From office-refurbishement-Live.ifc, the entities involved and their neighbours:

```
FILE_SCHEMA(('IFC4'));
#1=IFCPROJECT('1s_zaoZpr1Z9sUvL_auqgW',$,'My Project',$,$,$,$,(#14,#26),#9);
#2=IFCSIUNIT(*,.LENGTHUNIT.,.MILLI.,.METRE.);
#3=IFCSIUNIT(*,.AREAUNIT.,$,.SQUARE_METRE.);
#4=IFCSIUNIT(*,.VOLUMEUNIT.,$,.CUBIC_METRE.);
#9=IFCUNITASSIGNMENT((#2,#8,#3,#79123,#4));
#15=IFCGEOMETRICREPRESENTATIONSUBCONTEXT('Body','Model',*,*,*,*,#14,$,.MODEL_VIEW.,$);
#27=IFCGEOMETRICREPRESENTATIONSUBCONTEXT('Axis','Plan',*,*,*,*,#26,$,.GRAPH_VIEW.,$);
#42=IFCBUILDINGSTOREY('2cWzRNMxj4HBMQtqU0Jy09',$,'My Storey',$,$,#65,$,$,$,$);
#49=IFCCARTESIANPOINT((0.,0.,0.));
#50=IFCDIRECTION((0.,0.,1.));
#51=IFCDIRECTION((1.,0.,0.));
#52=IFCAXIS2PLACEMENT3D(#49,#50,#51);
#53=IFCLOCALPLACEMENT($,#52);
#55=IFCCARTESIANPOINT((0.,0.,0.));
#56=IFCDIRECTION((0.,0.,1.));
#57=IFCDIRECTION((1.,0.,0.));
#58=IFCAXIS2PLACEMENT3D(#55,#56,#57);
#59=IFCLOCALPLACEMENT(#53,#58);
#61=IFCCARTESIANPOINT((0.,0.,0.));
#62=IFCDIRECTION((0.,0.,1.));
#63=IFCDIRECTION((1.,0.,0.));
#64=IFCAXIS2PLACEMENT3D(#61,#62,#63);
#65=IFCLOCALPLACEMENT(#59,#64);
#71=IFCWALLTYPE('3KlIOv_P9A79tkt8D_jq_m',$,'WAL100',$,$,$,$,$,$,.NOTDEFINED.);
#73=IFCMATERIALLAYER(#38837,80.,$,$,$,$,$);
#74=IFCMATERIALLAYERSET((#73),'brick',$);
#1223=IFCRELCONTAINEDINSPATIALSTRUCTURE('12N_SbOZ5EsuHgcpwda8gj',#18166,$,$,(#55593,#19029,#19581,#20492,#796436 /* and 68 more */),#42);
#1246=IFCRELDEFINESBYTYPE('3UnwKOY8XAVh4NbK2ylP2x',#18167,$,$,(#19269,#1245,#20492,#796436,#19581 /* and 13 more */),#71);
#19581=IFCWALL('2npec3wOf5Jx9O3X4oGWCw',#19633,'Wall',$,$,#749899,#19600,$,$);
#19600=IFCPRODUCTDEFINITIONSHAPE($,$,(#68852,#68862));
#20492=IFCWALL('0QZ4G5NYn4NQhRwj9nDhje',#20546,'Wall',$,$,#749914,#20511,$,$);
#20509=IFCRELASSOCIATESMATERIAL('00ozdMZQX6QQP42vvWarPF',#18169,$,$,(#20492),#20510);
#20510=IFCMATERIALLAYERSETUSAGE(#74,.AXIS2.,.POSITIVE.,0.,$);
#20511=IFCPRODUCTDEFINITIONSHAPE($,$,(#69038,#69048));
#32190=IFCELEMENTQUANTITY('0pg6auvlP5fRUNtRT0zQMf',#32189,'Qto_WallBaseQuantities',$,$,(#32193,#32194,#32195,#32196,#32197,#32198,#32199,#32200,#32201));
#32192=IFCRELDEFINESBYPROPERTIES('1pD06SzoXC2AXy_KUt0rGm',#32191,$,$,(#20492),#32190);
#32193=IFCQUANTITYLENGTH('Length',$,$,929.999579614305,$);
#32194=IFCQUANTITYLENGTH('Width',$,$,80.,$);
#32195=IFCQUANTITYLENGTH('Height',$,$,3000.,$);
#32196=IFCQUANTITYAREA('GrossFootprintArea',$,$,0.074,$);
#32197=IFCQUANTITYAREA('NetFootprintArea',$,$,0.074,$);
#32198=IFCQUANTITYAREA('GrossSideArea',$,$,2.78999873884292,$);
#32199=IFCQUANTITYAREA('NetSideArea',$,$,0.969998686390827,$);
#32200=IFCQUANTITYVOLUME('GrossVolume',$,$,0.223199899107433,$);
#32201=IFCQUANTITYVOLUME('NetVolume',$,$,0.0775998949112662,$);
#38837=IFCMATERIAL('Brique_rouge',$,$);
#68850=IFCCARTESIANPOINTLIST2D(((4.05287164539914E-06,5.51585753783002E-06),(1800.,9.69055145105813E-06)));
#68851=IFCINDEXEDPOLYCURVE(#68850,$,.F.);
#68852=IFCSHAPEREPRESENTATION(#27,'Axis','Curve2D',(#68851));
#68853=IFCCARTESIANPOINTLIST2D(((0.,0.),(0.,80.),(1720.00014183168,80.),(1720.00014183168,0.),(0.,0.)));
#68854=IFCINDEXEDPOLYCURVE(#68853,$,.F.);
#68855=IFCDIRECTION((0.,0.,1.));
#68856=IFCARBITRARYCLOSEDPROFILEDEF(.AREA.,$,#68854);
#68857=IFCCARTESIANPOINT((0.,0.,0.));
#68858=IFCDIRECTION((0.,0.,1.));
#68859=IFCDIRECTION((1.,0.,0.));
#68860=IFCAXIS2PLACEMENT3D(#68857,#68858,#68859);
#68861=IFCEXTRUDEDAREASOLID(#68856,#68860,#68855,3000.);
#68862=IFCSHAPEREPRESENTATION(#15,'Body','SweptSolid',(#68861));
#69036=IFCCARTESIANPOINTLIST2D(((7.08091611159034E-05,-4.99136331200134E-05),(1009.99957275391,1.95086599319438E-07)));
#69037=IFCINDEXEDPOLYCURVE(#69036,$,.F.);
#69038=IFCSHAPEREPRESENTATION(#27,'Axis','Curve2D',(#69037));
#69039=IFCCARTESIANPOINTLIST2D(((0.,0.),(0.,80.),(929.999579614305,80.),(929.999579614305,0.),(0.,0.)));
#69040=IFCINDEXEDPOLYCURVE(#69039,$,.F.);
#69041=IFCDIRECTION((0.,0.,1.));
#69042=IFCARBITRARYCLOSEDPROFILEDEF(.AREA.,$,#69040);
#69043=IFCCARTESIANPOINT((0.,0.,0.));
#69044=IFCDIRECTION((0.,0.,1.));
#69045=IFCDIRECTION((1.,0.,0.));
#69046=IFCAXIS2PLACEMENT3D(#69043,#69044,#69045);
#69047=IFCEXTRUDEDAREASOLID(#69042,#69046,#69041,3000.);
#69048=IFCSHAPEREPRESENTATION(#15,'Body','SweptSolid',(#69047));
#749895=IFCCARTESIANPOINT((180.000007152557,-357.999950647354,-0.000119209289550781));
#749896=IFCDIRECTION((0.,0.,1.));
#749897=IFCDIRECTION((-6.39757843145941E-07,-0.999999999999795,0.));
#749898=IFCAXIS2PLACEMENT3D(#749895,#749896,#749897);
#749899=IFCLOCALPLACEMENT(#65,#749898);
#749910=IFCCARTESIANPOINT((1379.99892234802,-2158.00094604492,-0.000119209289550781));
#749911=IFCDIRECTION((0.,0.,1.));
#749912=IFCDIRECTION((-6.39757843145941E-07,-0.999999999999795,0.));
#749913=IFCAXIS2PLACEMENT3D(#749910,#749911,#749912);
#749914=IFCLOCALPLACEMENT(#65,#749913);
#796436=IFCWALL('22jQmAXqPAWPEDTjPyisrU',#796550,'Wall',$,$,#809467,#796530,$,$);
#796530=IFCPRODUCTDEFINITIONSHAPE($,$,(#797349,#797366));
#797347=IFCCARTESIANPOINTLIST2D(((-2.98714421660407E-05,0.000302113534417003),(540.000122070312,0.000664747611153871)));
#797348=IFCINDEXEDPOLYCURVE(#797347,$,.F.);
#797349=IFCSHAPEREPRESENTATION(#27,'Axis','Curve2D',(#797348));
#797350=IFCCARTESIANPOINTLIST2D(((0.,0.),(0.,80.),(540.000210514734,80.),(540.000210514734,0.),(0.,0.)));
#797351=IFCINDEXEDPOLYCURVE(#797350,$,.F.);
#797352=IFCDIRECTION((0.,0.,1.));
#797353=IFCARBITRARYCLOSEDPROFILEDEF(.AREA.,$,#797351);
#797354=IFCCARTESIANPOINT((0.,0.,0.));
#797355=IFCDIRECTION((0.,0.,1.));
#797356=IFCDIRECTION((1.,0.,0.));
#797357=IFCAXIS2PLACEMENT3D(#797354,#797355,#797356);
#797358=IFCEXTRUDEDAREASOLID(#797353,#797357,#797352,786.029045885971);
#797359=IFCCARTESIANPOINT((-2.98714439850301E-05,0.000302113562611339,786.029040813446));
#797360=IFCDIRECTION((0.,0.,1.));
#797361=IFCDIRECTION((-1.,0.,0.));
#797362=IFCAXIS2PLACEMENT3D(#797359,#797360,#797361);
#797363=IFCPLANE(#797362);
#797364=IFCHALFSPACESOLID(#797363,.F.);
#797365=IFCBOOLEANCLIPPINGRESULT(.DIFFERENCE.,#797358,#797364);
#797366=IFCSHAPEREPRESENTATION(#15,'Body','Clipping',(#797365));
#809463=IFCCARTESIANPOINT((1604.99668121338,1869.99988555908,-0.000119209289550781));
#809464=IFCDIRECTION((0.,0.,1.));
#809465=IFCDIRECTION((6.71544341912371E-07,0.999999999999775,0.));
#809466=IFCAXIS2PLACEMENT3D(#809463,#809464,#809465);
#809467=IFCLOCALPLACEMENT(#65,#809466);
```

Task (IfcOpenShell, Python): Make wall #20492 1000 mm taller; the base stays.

```python
import ifcopenshell
import ifcopenshell.api.pset
import ifcopenshell.geom
import ifcopenshell.util.element
import ifcopenshell.util.representation
import ifcopenshell.util.shape
import ifcopenshell.util.unit

model = ifcopenshell.open("office-refurbishement-Live.ifc")
unit_scale = ifcopenshell.util.unit.calculate_unit_scale(model)
area_scale = ifcopenshell.util.unit.calculate_unit_scale(model, "AREAUNIT")
volume_scale = ifcopenshell.util.unit.calculate_unit_scale(model, "VOLUMEUNIT")
settings = ifcopenshell.geom.settings()


def volume(element):
    """Net volume in cubic metres, openings subtracted."""
    shape = ifcopenshell.geom.create_shape(settings, element)
    return ifcopenshell.util.shape.get_volume(shape.geometry)


wall = model.by_id(20492)
before = volume(wall)

body = ifcopenshell.util.representation.get_representation(wall, "Model", "Body")
solid = body.Items[0]
old_height = solid.Depth
solid.Depth += 1 / unit_scale
after = volume(wall)
thickness = 0.08  # wall thickness in metres

# Update the stored height, areas and volumes.
qto = model.by_id(ifcopenshell.util.element.get_pset(wall, "Qto_WallBaseQuantities", should_inherit=False)["id"])
ifcopenshell.api.pset.edit_qto(model, qto=qto, properties={
    "Height": solid.Depth,
    "GrossSideArea": ifcopenshell.util.element.get_pset(wall, "Qto_WallBaseQuantities", "GrossSideArea") * solid.Depth / old_height,
    "NetSideArea": after / thickness / area_scale,
    "GrossVolume": ifcopenshell.util.element.get_pset(wall, "Qto_WallBaseQuantities", "GrossVolume") * solid.Depth / old_height,
    "NetVolume": after / volume_scale,
})

print(f"height {old_height:g} -> {solid.Depth:g}, volume {before:.3f} -> {after:.3f} m3")

model.write("office-refurbishement-Live_updated.ifc")
```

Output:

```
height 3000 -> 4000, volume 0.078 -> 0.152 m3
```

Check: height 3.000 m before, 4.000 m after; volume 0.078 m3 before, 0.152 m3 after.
